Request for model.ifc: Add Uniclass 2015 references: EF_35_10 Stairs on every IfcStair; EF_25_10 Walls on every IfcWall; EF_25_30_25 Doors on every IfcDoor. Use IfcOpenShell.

First a look at what the model holds.

```python
import ifcopenshell

model = ifcopenshell.open("model.ifc")
print(model.schema)
print("classifications:", [c.Name for c in model.by_type("IfcClassification")])
for ifc_class in ("IfcDoor", "IfcRoof", "IfcStair", "IfcWall", "IfcWindow"):
    print(ifc_class, len(model.by_type(ifc_class)))
```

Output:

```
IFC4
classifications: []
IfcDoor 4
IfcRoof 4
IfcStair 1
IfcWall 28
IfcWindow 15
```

```python
import ifcopenshell
import ifcopenshell.api.classification

model = ifcopenshell.open("model.ifc")

system = ifcopenshell.api.classification.add_classification(model, classification="Uniclass 2015")

codes = {
    "IfcStair": ("EF_35_10", "Stairs"),
    "IfcWall": ("EF_25_10", "Walls"),
    "IfcDoor": ("EF_25_30_25", "Doors"),
}
for ifc_class, (code, name) in codes.items():
    products = model.by_type(ifc_class)
    ifcopenshell.api.classification.add_reference(
        model, products=products, classification=system, identification=code, name=name
    )
    print(code, len(products))

model.write("model_updated.ifc")
```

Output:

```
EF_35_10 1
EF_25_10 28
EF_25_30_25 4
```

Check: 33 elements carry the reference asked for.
